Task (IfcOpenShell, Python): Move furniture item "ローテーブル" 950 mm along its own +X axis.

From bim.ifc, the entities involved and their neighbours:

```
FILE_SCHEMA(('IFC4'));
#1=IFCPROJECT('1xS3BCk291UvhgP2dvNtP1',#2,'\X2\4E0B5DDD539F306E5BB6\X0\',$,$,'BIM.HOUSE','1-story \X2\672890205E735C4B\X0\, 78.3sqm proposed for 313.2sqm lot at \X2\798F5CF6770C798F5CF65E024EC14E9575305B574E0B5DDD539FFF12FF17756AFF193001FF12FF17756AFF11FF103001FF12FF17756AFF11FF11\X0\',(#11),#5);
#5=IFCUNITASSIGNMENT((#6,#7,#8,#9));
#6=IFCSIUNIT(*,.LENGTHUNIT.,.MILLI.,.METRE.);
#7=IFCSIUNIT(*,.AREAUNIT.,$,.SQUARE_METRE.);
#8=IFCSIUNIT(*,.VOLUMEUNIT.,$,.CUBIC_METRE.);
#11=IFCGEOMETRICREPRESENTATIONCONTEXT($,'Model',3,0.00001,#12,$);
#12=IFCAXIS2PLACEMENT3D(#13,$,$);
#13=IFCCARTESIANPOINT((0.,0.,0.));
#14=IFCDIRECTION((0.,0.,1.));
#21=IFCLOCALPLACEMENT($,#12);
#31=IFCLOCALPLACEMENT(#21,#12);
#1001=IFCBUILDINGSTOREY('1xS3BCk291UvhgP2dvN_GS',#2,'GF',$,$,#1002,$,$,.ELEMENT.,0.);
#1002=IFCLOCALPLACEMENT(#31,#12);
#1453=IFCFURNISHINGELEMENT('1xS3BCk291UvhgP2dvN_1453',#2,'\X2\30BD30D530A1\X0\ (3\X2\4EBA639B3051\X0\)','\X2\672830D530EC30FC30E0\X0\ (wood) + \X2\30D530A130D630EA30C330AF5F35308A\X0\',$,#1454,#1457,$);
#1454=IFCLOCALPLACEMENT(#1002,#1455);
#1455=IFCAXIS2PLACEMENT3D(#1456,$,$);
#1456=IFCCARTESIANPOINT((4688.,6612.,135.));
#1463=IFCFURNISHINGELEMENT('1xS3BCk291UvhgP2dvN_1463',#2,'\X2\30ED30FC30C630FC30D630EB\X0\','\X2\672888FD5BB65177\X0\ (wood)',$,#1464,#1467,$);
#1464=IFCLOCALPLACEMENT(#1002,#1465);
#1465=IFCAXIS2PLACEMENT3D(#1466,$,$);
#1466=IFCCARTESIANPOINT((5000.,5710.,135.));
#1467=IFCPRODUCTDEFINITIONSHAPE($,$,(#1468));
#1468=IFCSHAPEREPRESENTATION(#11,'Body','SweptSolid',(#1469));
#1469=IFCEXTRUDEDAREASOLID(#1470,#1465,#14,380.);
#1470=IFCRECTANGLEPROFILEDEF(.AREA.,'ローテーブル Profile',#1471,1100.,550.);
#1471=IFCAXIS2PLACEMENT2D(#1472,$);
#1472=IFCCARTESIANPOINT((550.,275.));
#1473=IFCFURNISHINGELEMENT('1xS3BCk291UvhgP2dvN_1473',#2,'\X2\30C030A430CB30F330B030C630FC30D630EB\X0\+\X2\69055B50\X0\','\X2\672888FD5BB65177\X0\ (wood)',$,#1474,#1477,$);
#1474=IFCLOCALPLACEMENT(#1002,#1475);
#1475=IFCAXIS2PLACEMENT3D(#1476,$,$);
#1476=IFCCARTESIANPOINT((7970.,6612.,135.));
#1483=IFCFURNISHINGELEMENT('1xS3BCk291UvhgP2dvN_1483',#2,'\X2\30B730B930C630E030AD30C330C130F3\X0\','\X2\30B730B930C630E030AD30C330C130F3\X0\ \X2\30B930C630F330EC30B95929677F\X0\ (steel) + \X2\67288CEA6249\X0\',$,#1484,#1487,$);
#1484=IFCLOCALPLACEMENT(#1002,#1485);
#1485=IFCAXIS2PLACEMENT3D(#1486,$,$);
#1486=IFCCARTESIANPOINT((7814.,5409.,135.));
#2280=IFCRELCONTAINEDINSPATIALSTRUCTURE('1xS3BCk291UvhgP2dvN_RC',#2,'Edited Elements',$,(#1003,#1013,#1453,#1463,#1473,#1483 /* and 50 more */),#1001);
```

```python
import ifcopenshell
import ifcopenshell.api.geometry
import ifcopenshell.util.placement

model = ifcopenshell.open("bim.ifc")

item = model.by_guid("1xS3BCk291UvhgP2dvN_1463")
matrix = ifcopenshell.util.placement.get_local_placement(item.ObjectPlacement)
matrix[:3, 3] += matrix[:3, 0] * 950.0
ifcopenshell.api.geometry.edit_object_placement(model, product=item, matrix=matrix, is_si=False)

print(ifcopenshell.util.placement.get_local_placement(item.ObjectPlacement).round(3) + 0.0)

model.write("bim_updated.ifc")
```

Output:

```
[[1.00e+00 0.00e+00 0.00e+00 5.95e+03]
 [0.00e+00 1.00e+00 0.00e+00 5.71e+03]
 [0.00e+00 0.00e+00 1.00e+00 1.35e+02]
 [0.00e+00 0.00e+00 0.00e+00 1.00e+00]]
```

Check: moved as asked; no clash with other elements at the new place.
